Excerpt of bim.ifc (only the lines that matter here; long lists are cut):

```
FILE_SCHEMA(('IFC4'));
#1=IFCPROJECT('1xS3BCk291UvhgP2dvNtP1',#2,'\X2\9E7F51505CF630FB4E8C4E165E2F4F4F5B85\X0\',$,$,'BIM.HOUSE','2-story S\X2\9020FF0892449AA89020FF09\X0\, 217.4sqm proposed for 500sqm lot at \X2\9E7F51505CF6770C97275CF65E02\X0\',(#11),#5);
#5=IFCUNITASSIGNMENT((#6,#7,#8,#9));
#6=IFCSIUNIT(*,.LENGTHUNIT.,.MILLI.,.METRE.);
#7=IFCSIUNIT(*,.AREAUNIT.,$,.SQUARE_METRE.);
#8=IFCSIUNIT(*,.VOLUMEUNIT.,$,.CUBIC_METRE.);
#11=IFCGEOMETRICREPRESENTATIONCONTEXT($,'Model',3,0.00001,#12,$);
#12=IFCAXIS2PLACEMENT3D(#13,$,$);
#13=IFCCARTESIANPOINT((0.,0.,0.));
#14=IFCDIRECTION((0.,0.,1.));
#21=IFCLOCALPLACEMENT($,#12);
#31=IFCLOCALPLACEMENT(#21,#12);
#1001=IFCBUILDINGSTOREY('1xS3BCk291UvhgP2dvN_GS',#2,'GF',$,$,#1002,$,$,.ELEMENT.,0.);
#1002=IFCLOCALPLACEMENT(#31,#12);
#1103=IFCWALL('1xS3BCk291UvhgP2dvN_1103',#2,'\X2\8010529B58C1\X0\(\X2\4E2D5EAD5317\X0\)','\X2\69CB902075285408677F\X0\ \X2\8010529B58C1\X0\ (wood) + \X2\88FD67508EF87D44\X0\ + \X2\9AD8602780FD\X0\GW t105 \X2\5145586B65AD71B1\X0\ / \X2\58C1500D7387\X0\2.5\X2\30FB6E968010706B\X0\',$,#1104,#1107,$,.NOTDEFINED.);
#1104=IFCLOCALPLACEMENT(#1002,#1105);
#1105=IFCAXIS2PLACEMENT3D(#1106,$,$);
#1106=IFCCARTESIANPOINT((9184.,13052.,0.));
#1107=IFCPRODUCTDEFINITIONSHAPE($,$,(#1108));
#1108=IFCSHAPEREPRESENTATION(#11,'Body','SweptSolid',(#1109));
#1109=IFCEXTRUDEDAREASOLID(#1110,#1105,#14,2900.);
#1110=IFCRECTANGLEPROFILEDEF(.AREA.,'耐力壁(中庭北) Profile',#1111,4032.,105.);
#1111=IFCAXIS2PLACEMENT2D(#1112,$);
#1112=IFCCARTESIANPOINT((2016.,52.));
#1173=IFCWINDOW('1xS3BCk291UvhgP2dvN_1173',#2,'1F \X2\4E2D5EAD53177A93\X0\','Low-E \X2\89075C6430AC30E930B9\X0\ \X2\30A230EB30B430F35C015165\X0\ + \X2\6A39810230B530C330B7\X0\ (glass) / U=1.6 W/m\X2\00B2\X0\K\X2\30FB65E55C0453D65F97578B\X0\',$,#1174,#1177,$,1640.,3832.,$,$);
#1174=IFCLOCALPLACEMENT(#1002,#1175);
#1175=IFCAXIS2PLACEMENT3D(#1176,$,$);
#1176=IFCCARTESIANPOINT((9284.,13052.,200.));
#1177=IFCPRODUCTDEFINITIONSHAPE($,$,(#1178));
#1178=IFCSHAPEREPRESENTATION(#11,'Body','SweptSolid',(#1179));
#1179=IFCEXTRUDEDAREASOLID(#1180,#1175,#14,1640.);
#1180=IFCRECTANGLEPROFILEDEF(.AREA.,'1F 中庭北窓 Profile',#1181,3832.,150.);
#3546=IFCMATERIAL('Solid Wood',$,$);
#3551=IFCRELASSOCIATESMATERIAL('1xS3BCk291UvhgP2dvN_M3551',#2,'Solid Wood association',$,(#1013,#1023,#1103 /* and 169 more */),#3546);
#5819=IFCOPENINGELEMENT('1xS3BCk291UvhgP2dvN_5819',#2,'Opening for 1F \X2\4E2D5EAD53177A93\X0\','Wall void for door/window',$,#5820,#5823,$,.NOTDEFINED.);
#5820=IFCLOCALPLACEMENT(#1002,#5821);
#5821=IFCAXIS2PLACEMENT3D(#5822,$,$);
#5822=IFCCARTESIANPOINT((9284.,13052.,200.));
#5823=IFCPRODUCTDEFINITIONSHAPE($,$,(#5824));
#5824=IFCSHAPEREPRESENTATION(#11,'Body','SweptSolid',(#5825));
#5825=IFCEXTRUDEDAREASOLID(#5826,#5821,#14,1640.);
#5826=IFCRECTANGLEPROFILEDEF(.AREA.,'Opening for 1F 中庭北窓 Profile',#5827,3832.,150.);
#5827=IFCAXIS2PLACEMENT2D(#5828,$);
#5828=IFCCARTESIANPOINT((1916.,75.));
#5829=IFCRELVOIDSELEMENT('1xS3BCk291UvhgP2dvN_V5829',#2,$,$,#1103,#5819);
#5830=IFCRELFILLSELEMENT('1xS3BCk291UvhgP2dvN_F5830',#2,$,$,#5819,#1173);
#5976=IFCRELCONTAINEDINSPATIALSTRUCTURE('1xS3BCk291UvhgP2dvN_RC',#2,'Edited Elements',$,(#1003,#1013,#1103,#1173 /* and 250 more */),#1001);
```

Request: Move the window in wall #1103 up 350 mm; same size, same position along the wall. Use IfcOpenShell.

```python
import numpy as np
import ifcopenshell
import ifcopenshell.api.geometry
import ifcopenshell.util.placement
import ifcopenshell.util.unit

model = ifcopenshell.open("bim.ifc")
unit_scale = ifcopenshell.util.unit.calculate_unit_scale(model)

window = model.by_guid("1xS3BCk291UvhgP2dvN_1173")
opening = window.FillsVoids[0].RelatingOpeningElement
dz = 0.35 / unit_scale

shift = np.array([0.0, 0.0, dz])
# The window is not placed relative to its opening, so move both.
for product in (opening, window):
    matrix = ifcopenshell.util.placement.get_local_placement(product.ObjectPlacement)
    matrix[:3, 3] += shift
    ifcopenshell.api.geometry.edit_object_placement(model, product=product, matrix=matrix, is_si=False)

print(f"moved by {dz * unit_scale:+.3f} m")

model.write("bim-out.ifc")
```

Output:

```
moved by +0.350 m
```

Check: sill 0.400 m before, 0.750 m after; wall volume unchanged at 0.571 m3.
